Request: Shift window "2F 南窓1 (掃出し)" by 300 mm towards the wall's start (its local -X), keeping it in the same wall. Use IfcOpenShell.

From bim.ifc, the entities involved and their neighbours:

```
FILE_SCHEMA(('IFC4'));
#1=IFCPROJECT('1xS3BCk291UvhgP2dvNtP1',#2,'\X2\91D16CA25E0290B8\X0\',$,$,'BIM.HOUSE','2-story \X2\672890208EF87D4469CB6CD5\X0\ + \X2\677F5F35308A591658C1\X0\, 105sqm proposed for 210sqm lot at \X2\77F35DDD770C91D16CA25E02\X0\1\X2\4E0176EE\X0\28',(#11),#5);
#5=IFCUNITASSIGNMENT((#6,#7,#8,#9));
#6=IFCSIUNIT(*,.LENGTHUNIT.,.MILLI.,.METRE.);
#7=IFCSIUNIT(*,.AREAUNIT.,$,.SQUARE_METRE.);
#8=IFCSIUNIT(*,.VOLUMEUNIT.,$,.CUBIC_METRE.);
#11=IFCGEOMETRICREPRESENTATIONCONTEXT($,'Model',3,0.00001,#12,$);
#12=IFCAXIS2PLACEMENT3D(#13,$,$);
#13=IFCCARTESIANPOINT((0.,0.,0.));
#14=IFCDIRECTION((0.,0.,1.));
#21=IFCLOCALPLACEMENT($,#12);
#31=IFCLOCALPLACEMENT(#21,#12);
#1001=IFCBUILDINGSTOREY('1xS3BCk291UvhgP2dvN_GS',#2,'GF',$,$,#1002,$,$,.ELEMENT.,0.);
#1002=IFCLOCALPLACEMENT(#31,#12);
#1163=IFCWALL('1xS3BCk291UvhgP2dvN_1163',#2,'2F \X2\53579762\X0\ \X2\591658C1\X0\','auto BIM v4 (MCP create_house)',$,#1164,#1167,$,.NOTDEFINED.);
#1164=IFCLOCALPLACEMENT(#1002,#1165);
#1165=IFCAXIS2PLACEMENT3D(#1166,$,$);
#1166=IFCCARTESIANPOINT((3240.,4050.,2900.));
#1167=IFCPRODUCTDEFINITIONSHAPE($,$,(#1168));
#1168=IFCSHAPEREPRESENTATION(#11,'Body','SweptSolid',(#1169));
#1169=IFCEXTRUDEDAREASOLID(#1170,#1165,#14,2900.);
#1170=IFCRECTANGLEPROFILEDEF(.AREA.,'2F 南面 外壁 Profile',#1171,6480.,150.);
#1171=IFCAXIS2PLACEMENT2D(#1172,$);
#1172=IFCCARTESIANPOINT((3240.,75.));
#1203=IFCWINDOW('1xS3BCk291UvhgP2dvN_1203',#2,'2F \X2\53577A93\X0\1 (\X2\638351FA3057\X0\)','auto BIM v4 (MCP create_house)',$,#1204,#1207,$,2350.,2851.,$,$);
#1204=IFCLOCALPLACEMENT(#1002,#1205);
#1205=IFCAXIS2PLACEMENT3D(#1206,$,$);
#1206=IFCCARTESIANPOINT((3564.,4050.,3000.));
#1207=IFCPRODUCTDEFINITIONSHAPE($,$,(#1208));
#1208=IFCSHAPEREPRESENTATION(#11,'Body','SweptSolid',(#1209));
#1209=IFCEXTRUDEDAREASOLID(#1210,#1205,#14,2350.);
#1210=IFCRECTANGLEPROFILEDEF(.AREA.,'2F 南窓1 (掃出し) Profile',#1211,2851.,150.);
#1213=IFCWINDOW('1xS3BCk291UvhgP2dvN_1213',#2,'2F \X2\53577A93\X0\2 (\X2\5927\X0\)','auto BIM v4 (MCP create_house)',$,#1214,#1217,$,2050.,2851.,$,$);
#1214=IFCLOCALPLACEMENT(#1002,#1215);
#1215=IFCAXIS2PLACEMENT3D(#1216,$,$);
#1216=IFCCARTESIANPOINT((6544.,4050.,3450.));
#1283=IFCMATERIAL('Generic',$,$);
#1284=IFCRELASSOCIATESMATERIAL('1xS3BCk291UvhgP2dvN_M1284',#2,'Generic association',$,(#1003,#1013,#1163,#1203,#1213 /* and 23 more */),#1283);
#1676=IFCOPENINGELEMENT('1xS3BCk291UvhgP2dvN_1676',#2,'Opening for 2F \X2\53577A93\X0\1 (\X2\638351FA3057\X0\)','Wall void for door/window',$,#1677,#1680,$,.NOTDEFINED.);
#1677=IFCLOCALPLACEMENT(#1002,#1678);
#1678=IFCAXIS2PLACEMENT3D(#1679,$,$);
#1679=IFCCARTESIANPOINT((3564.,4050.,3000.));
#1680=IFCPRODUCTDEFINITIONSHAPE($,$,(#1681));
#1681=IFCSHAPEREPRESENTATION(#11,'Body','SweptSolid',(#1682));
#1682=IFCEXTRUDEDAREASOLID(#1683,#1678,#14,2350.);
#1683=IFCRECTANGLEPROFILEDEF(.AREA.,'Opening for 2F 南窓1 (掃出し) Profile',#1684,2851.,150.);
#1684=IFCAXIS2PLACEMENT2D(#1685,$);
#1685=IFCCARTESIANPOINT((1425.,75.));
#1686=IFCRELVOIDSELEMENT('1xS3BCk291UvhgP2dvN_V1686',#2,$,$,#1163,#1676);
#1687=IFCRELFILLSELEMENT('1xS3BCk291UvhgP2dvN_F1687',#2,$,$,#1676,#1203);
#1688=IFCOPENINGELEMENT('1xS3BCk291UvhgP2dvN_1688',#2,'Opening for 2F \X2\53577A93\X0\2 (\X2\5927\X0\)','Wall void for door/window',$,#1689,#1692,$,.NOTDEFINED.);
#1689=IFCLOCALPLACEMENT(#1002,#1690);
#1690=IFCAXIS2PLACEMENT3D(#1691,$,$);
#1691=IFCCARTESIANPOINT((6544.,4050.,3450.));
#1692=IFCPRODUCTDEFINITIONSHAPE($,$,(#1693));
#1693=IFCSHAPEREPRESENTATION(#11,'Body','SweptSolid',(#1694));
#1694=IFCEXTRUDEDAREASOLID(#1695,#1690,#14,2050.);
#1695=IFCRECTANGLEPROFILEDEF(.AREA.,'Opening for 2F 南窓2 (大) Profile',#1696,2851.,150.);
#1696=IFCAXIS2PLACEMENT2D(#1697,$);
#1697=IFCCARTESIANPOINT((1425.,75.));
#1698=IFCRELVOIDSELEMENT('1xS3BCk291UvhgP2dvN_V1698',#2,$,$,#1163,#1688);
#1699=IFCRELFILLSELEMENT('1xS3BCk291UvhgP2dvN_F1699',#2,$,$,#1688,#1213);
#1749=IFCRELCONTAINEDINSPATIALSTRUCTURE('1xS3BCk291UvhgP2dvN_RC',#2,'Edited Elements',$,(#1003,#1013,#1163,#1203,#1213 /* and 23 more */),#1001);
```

```python
import ifcopenshell
import ifcopenshell.api.geometry
import ifcopenshell.util.placement

model = ifcopenshell.open("bim.ifc")

window = model.by_id(1203)
opening = window.FillsVoids[0].RelatingOpeningElement
wall = opening.VoidsElements[0].RelatingBuildingElement

wall_matrix = ifcopenshell.util.placement.get_local_placement(wall.ObjectPlacement)
shift = wall_matrix[:3, 0] * -300.0
before = ifcopenshell.util.placement.get_local_placement(window.ObjectPlacement)[:3, 3].copy()

# The window is not placed relative to its opening, so move both.
for product in (opening, window):
    matrix = ifcopenshell.util.placement.get_local_placement(product.ObjectPlacement)
    matrix[:3, 3] += shift
    ifcopenshell.api.geometry.edit_object_placement(model, product=product, matrix=matrix, is_si=False)

after = ifcopenshell.util.placement.get_local_placement(window.ObjectPlacement)[:3, 3]
print("window moved by", (after - before).round(3) + 0.0)

model.write("bim_edited.ifc")
```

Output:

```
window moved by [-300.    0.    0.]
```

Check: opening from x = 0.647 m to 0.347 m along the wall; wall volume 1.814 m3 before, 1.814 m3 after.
